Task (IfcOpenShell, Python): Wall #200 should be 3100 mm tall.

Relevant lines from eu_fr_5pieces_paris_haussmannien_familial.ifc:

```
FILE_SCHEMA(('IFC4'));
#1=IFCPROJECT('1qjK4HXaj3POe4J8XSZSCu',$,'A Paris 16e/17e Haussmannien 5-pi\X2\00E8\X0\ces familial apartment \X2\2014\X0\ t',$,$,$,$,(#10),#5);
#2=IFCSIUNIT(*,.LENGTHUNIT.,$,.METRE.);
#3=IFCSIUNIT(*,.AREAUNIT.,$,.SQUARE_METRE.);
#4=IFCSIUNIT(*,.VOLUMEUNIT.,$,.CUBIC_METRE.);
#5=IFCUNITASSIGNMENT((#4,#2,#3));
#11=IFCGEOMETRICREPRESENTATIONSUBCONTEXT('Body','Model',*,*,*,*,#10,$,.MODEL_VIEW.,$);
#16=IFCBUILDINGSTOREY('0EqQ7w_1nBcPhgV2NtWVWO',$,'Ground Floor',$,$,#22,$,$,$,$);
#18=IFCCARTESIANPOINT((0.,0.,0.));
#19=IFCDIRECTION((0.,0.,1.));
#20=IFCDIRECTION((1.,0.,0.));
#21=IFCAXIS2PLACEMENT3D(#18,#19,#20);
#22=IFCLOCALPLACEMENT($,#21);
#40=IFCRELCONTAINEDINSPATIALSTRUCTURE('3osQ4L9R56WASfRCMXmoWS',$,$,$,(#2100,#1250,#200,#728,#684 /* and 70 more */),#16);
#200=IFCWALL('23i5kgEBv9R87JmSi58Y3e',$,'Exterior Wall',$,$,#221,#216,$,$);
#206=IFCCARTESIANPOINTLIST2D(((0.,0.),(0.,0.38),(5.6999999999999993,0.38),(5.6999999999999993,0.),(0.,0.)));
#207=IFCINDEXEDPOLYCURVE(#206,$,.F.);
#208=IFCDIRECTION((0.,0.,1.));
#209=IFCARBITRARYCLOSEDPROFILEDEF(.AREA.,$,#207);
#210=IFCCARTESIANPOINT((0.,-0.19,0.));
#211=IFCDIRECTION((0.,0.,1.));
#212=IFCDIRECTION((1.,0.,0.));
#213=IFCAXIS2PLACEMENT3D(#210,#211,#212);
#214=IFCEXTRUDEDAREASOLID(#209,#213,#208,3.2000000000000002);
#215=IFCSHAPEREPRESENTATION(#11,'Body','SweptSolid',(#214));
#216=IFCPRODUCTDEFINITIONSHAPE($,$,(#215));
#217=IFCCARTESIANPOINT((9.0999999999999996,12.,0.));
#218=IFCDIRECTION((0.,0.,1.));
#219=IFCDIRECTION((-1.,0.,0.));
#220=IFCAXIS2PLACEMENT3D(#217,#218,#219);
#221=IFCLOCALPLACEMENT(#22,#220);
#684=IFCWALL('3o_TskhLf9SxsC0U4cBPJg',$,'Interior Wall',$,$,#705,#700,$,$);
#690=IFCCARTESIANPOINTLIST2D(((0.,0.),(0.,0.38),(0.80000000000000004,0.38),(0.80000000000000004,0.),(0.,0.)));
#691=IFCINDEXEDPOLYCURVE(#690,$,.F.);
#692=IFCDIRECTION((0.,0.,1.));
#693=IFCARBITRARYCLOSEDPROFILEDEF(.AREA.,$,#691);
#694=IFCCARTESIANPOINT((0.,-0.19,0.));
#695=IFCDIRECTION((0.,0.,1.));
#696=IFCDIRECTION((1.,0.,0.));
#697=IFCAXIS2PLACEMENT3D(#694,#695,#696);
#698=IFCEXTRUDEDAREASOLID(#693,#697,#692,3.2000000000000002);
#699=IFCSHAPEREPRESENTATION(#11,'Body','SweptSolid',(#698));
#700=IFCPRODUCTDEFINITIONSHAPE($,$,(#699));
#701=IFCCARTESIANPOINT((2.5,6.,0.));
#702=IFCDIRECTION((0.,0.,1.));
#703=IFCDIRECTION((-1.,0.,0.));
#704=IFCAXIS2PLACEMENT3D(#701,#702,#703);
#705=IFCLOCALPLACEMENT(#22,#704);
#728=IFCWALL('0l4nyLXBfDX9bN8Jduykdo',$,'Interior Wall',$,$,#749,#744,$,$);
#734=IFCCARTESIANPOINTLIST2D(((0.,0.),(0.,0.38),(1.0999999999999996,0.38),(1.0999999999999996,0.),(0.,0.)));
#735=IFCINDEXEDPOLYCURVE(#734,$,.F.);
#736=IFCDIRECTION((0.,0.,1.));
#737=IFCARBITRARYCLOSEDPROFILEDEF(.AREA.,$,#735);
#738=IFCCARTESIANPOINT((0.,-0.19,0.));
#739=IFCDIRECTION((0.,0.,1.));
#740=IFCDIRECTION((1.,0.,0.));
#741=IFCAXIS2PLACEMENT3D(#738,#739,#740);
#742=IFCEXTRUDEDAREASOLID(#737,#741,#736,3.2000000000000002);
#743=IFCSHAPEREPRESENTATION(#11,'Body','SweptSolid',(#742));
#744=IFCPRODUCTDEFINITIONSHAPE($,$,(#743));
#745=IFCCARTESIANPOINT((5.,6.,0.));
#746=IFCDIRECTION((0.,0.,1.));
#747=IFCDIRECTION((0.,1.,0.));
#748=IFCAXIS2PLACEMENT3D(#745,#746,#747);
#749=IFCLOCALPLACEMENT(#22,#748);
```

```python
import ifcopenshell
import ifcopenshell.geom
import ifcopenshell.util.representation
import ifcopenshell.util.shape
import ifcopenshell.util.unit

model = ifcopenshell.open("eu_fr_5pieces_paris_haussmannien_familial.ifc")
unit_scale = ifcopenshell.util.unit.calculate_unit_scale(model)
settings = ifcopenshell.geom.settings()


def volume(element):
    """Net volume in cubic metres, openings subtracted."""
    shape = ifcopenshell.geom.create_shape(settings, element)
    return ifcopenshell.util.shape.get_volume(shape.geometry)


wall = model.by_id(200)
before = volume(wall)

body = ifcopenshell.util.representation.get_representation(wall, "Model", "Body")
solid = body.Items[0]
old_height = solid.Depth
solid.Depth = 3.1 / unit_scale
after = volume(wall)

print(f"height {old_height:g} -> {solid.Depth:g}, volume {before:.3f} -> {after:.3f} m3")

model.write("eu_fr_5pieces_paris_haussmannien_familial_v2.ifc")
```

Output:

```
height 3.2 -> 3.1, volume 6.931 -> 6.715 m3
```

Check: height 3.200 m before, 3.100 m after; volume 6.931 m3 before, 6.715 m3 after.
